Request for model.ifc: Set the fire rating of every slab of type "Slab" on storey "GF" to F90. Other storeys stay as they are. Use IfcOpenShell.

First a look at what the model holds.

```python
import ifcopenshell
import ifcopenshell.util.element

model = ifcopenshell.open("model.ifc")
print(model.schema)
storey = next(s for s in model.by_type("IfcBuildingStorey") if s.Name == "GF")
slabs = [e for e in ifcopenshell.util.element.get_decomposition(storey) if e.is_a("IfcSlab")]
seen = {}
for e in slabs:
    element_type = ifcopenshell.util.element.get_type(e)
    key = (element_type.Name if element_type != e and element_type else None, ifcopenshell.util.element.get_pset(e, "Pset_SlabCommon", "FireRating"))
    seen[key] = seen.get(key, 0) + 1
for (name, value), count in sorted(seen.items(), key=str):
    print(count, "x", name, "|", value)
```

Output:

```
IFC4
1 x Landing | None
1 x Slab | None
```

```python
import ifcopenshell
import ifcopenshell.api.pset
import ifcopenshell.util.element

model = ifcopenshell.open("model.ifc")

storey = next(s for s in model.by_type("IfcBuildingStorey") if s.Name == "GF")
slabs = [e for e in ifcopenshell.util.element.get_decomposition(storey) if e.is_a("IfcSlab")]

count = 0
for e in slabs:
    element_type = ifcopenshell.util.element.get_type(e)
    if element_type in (None, e) or element_type.Name != "Slab":
        continue
    # add_pset returns the element's existing set when there is one.
    pset = ifcopenshell.api.pset.add_pset(model, product=e, name="Pset_SlabCommon")
    ifcopenshell.api.pset.edit_pset(model, pset=pset, properties={"FireRating": "F90"})
    count += 1

print(count, "slabs updated")

model.write("model_rev.ifc")
```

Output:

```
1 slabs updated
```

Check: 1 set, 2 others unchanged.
